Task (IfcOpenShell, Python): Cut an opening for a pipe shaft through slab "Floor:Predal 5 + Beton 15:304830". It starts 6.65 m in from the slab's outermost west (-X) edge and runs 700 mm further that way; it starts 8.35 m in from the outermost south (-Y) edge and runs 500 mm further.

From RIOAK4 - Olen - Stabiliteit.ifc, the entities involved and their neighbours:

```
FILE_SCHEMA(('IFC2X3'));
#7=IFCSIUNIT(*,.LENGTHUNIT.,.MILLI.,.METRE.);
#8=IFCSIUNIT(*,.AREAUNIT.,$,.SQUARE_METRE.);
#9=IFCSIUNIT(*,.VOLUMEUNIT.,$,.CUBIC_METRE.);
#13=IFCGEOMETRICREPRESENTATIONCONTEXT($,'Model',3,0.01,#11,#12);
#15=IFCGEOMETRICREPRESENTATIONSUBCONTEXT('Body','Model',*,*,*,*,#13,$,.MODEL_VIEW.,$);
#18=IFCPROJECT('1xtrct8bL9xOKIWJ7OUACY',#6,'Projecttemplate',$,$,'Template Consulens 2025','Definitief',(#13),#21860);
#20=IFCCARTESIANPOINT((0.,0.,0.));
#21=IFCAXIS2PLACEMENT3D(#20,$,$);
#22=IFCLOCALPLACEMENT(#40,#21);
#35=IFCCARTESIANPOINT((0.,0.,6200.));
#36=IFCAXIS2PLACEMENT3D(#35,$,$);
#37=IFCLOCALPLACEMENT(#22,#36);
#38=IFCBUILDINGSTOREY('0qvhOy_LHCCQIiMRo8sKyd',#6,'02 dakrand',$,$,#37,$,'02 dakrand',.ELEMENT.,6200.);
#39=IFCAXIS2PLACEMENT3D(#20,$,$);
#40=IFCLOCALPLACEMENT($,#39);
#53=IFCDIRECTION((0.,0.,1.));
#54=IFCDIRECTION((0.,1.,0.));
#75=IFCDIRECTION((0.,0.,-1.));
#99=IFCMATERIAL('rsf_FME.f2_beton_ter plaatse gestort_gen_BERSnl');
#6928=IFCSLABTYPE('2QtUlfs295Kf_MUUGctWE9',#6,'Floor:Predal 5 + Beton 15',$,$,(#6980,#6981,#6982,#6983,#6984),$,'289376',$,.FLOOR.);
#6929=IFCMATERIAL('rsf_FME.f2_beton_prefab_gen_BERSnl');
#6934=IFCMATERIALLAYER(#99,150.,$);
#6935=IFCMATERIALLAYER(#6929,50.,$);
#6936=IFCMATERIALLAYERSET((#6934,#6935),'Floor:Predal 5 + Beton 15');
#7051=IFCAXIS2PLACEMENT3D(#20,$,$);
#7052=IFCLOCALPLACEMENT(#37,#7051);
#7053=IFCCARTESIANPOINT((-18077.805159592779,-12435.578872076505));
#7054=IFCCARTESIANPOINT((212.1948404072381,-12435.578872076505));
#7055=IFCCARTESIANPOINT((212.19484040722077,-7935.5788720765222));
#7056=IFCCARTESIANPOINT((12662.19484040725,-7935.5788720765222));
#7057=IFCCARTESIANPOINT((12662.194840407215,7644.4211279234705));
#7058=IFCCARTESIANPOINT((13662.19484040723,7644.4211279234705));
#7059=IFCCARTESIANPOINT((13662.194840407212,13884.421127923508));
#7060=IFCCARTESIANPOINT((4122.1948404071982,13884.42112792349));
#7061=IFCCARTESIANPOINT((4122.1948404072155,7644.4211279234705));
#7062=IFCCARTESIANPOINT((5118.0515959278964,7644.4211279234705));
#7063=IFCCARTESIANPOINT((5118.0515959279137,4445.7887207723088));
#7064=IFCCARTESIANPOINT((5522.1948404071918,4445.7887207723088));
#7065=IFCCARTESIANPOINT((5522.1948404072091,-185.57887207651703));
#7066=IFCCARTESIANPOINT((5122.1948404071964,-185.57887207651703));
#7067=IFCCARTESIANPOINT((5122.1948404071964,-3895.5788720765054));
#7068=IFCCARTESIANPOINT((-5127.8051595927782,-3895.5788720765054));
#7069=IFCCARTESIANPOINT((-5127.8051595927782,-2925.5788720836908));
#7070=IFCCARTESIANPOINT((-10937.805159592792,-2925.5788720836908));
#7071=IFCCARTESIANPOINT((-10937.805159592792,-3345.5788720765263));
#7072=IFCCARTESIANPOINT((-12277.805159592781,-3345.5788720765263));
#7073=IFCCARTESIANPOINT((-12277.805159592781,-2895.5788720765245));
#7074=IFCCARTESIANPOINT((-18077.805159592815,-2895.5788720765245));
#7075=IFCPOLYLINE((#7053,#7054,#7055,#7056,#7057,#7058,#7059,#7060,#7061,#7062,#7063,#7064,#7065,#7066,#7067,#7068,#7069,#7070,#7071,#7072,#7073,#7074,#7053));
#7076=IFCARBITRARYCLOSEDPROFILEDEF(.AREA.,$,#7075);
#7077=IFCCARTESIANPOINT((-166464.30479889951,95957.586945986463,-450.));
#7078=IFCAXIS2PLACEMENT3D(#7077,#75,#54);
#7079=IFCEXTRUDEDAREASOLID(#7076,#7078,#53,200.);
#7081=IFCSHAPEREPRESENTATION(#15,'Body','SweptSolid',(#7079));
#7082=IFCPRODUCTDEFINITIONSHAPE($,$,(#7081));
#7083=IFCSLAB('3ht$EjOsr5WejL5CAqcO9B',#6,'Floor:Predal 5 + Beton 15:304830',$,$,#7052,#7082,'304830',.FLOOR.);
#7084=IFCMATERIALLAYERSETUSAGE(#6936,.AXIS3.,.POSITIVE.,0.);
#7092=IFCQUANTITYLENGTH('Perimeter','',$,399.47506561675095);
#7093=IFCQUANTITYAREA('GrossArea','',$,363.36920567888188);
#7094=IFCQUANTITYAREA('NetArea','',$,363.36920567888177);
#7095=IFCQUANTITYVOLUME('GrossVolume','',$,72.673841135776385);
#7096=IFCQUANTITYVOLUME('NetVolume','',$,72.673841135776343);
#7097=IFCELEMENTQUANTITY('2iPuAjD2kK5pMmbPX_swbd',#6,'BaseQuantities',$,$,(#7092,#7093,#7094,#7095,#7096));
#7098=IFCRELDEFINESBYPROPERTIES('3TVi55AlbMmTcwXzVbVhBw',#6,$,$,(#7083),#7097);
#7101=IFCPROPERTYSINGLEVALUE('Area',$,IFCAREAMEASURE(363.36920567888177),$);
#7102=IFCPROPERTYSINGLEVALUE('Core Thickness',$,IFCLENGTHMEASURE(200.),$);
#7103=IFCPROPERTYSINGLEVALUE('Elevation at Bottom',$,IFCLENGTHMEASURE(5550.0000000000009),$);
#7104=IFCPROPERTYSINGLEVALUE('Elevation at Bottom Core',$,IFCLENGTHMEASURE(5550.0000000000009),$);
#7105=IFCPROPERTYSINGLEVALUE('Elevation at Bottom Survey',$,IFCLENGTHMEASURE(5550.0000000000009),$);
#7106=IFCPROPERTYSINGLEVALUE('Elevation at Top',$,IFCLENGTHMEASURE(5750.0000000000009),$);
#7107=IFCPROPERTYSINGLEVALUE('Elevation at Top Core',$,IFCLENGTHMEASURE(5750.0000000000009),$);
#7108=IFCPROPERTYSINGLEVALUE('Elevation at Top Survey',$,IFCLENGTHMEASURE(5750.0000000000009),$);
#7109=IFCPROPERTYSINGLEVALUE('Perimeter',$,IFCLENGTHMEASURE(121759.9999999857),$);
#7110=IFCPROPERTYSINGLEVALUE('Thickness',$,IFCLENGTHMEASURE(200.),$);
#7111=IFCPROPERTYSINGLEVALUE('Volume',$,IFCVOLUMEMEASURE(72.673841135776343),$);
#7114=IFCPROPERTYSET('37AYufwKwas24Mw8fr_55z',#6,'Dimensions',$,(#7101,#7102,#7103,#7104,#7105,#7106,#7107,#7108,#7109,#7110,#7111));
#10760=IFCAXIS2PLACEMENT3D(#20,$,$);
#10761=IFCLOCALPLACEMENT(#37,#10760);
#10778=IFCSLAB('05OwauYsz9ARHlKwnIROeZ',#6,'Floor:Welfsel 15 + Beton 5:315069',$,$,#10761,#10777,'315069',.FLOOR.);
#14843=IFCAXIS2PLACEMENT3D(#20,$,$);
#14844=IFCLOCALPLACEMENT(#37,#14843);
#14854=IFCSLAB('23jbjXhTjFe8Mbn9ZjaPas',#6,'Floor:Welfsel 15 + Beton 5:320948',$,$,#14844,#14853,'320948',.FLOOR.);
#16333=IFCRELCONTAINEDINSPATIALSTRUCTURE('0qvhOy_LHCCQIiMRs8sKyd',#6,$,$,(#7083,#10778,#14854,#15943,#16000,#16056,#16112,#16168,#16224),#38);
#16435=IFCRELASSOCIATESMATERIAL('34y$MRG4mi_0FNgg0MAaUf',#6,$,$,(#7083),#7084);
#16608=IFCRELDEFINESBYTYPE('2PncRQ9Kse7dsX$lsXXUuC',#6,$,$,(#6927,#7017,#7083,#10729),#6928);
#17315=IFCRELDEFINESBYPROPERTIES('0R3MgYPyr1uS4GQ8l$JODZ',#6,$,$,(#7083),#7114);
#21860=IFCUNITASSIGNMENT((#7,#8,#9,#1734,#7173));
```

```python
import numpy as np
import ifcopenshell
import ifcopenshell.api.feature
import ifcopenshell.api.geometry
import ifcopenshell.api.pset
import ifcopenshell.api.root
import ifcopenshell.geom
import ifcopenshell.util.element
import ifcopenshell.util.placement
import ifcopenshell.util.representation
import ifcopenshell.util.shape
import ifcopenshell.util.unit

model = ifcopenshell.open("RIOAK4 - Olen - Stabiliteit.ifc")
unit_scale = ifcopenshell.util.unit.calculate_unit_scale(model)
area_scale = ifcopenshell.util.unit.calculate_unit_scale(model, "AREAUNIT")
volume_scale = ifcopenshell.util.unit.calculate_unit_scale(model, "VOLUMEUNIT")
settings = ifcopenshell.geom.settings()


def volume(element):
    """Net volume in cubic metres, openings subtracted."""
    shape = ifcopenshell.geom.create_shape(settings, element)
    return ifcopenshell.util.shape.get_volume(shape.geometry)


slab = model.by_guid("3ht$EjOsr5WejL5CAqcO9B")
before = volume(slab)

# Extent in the slab's own axes, in metres. The edges named are its -X and -Y sides.
slab_shape = ifcopenshell.geom.create_shape(settings, slab)
vertices = ifcopenshell.util.shape.get_vertices(slab_shape.geometry)
x_min, y_min, bottom = vertices.min(axis=0)
top = vertices[:, 2].max()

opening = ifcopenshell.api.root.create_entity(model, ifc_class="IfcOpeningElement", name="Pipe shaft opening")
context = ifcopenshell.util.representation.get_context(model, "Model", "Body", "MODEL_VIEW")
width, depth = 0.7, 0.5
outline = [(0.0, 0.0), (width, 0.0), (width, depth), (0.0, depth), (0.0, 0.0)]
# Overshoot both faces by 50 mm so the cut is clean.
shape = ifcopenshell.api.geometry.add_slab_representation(
    model, context=context, depth=top - bottom + 0.1, polyline=outline
)
ifcopenshell.api.geometry.assign_representation(model, product=opening, representation=shape)

matrix = ifcopenshell.util.placement.get_local_placement(slab.ObjectPlacement)
matrix[:, 3] = matrix @ np.append(np.array([x_min + 6.65, y_min + 8.35, bottom - 0.05]) / unit_scale, 1.0)
ifcopenshell.api.geometry.edit_object_placement(model, product=opening, matrix=matrix, is_si=False)
ifcopenshell.api.feature.add_feature(model, feature=opening, element=slab)

after = volume(slab)

# Update the slab's stored quantities.
qto = model.by_id(ifcopenshell.util.element.get_pset(slab, "BaseQuantities", should_inherit=False)["id"])
ifcopenshell.api.pset.edit_qto(model, qto=qto, properties={
    "NetArea": after / (top - bottom) / area_scale,
    "NetVolume": after / volume_scale,
})
pset = model.by_id(ifcopenshell.util.element.get_pset(slab, "Dimensions", should_inherit=False)["id"])
ifcopenshell.api.pset.edit_pset(model, pset=pset, properties={
    "Area": model.create_entity("IfcAreaMeasure", after / (top - bottom) / area_scale),
    "Volume": model.create_entity("IfcVolumeMeasure", after / volume_scale),
})

print(f"slab volume {before:.3f} -> {after:.3f} m3")

model.write("RIOAK4 - Olen - Stabiliteit-out.ifc")
```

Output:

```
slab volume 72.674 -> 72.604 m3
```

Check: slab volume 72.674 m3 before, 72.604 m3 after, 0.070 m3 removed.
